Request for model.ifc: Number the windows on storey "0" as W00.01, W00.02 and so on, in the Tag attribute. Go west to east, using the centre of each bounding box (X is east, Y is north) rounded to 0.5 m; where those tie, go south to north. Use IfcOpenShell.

First a look at what the model holds.

```python
import ifcopenshell
import ifcopenshell.util.element
import ifcopenshell.util.placement

model = ifcopenshell.open("model.ifc")
print(model.schema)
storey = next(s for s in model.by_type("IfcBuildingStorey") if s.Name == "0")
windows = [e for e in ifcopenshell.util.element.get_decomposition(storey) if e.is_a("IfcWindow")]
for e in sorted(windows, key=lambda e: e.id()):
    origin = ifcopenshell.util.placement.get_local_placement(e.ObjectPlacement)[:3, 3]
    print(e.id(), e.Tag, e.Name, origin.round(2) + 0.0, sep=" | ")
```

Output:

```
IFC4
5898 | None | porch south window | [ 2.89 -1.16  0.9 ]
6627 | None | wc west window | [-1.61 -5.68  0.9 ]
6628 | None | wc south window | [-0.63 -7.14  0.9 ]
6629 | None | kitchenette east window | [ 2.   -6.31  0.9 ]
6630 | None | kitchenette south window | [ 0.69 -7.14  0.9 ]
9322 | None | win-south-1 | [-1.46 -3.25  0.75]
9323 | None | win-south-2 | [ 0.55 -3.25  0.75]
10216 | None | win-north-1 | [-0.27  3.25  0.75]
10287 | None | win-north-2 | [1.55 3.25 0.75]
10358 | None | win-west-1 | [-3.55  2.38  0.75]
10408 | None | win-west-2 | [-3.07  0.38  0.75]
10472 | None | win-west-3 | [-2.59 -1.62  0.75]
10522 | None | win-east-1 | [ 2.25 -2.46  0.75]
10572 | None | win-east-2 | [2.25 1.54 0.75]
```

```python
import ifcopenshell
import ifcopenshell.geom
import ifcopenshell.util.element
import ifcopenshell.util.shape

model = ifcopenshell.open("model.ifc")
settings = ifcopenshell.geom.settings()
settings.set("use-world-coords", True)


def centre(element):
    shape = ifcopenshell.geom.create_shape(settings, element)
    return ifcopenshell.util.shape.get_bbox_centroid(shape.geometry)


storey = next(s for s in model.by_type("IfcBuildingStorey") if s.Name == "0")
windows = [e for e in ifcopenshell.util.element.get_decomposition(storey) if e.is_a("IfcWindow")]

# Insertion points can sit at a corner or the storey origin, so sort by the geometry (in metres).
centres = {e: centre(e) for e in windows}
windows.sort(key=lambda e: (round(centres[e][0] / 0.5), centres[e][1]))

for i, e in enumerate(windows, start=1):
    number = f"W00.{i:02d}"
    e.Tag = number
    print(e.id(), number)

model.write("model_updated.ifc")
```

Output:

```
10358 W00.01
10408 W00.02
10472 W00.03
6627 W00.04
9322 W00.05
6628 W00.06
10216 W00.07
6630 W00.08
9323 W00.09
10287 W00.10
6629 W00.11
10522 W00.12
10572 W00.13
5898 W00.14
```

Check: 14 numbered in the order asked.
